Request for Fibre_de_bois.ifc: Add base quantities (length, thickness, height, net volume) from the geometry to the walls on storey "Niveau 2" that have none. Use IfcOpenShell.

First a look at what the model holds.

```python
import ifcopenshell
import ifcopenshell.util.element
import ifcopenshell.util.unit

model = ifcopenshell.open("Fibre_de_bois.ifc")
print(model.schema)
for unit_type in ("LENGTHUNIT", "AREAUNIT", "VOLUMEUNIT"):
    print(unit_type, ifcopenshell.util.unit.calculate_unit_scale(model, unit_type))
storey = next(s for s in model.by_type("IfcBuildingStorey") if s.Name == "Niveau 2")
walls = [e for e in ifcopenshell.util.element.get_decomposition(storey) if e.is_a("IfcWall")]
for e in sorted(walls, key=lambda e: e.id()):
    print(e.id(), e.is_a(), e.Name, list(ifcopenshell.util.element.get_psets(e, qtos_only=True)), sep=" | ")
```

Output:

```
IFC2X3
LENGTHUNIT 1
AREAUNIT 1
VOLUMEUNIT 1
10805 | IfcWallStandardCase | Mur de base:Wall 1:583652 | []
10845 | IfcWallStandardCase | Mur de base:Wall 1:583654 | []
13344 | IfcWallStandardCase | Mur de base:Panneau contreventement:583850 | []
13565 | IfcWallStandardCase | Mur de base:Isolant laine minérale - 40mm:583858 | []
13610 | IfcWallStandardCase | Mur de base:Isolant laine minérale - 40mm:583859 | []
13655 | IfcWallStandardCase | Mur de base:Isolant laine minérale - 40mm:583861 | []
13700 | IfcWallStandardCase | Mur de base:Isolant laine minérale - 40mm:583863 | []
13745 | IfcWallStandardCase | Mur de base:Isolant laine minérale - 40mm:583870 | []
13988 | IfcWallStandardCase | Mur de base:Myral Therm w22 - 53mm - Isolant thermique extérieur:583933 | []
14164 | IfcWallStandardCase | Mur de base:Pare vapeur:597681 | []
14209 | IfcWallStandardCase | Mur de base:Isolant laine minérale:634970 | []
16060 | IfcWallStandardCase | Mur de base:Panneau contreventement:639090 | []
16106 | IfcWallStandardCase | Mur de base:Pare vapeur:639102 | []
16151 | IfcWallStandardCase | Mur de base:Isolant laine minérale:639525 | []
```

```python
import ifcopenshell
import ifcopenshell.api.pset
import ifcopenshell.geom
import ifcopenshell.util.element
import ifcopenshell.util.shape
import ifcopenshell.util.unit

model = ifcopenshell.open("Fibre_de_bois.ifc")
unit_scale = ifcopenshell.util.unit.calculate_unit_scale(model)
volume_scale = ifcopenshell.util.unit.calculate_unit_scale(model, "VOLUMEUNIT")
settings = ifcopenshell.geom.settings()

storey = next(s for s in model.by_type("IfcBuildingStorey") if s.Name == "Niveau 2")
walls = [e for e in ifcopenshell.util.element.get_decomposition(storey) if e.is_a("IfcWall")]

for e in sorted(walls, key=lambda e: e.id()):
    if ifcopenshell.util.element.get_psets(e, qtos_only=True, should_inherit=False):
        continue
    # Geometry comes back in metres, in the element's own axes.
    shape = ifcopenshell.geom.create_shape(settings, e)
    values = {
        "Length": ifcopenshell.util.shape.get_x(shape.geometry) / unit_scale,
        "Width": ifcopenshell.util.shape.get_y(shape.geometry) / unit_scale,
        "Height": ifcopenshell.util.shape.get_z(shape.geometry) / unit_scale,
        "NetVolume": ifcopenshell.util.shape.get_volume(shape.geometry) / volume_scale,
    }
    qto = ifcopenshell.api.pset.add_qto(model, product=e, name="BaseQuantities")
    ifcopenshell.api.pset.edit_qto(model, qto=qto, properties=values)
    print(e.id(), {k: round(v, 3) for k, v in values.items()})

model.write("Fibre_de_bois_rev.ifc")
```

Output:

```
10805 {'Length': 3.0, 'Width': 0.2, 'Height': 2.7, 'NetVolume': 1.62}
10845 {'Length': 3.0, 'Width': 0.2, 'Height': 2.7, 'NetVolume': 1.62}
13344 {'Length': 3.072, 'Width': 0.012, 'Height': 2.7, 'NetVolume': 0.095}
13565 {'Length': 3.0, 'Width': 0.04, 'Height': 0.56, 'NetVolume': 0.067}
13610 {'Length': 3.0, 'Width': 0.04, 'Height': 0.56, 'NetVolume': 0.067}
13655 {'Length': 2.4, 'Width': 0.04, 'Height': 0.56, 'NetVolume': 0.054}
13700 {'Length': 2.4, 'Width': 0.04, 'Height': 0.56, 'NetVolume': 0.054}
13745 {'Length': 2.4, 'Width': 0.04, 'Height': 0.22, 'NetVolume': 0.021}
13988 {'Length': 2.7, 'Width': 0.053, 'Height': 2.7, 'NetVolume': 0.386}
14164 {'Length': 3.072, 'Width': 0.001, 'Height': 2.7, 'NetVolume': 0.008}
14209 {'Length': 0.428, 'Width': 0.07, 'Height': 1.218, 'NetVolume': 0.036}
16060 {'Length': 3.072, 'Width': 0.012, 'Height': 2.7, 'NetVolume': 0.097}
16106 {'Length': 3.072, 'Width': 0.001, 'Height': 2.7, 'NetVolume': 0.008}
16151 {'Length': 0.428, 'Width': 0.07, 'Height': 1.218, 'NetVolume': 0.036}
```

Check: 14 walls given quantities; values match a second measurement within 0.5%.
